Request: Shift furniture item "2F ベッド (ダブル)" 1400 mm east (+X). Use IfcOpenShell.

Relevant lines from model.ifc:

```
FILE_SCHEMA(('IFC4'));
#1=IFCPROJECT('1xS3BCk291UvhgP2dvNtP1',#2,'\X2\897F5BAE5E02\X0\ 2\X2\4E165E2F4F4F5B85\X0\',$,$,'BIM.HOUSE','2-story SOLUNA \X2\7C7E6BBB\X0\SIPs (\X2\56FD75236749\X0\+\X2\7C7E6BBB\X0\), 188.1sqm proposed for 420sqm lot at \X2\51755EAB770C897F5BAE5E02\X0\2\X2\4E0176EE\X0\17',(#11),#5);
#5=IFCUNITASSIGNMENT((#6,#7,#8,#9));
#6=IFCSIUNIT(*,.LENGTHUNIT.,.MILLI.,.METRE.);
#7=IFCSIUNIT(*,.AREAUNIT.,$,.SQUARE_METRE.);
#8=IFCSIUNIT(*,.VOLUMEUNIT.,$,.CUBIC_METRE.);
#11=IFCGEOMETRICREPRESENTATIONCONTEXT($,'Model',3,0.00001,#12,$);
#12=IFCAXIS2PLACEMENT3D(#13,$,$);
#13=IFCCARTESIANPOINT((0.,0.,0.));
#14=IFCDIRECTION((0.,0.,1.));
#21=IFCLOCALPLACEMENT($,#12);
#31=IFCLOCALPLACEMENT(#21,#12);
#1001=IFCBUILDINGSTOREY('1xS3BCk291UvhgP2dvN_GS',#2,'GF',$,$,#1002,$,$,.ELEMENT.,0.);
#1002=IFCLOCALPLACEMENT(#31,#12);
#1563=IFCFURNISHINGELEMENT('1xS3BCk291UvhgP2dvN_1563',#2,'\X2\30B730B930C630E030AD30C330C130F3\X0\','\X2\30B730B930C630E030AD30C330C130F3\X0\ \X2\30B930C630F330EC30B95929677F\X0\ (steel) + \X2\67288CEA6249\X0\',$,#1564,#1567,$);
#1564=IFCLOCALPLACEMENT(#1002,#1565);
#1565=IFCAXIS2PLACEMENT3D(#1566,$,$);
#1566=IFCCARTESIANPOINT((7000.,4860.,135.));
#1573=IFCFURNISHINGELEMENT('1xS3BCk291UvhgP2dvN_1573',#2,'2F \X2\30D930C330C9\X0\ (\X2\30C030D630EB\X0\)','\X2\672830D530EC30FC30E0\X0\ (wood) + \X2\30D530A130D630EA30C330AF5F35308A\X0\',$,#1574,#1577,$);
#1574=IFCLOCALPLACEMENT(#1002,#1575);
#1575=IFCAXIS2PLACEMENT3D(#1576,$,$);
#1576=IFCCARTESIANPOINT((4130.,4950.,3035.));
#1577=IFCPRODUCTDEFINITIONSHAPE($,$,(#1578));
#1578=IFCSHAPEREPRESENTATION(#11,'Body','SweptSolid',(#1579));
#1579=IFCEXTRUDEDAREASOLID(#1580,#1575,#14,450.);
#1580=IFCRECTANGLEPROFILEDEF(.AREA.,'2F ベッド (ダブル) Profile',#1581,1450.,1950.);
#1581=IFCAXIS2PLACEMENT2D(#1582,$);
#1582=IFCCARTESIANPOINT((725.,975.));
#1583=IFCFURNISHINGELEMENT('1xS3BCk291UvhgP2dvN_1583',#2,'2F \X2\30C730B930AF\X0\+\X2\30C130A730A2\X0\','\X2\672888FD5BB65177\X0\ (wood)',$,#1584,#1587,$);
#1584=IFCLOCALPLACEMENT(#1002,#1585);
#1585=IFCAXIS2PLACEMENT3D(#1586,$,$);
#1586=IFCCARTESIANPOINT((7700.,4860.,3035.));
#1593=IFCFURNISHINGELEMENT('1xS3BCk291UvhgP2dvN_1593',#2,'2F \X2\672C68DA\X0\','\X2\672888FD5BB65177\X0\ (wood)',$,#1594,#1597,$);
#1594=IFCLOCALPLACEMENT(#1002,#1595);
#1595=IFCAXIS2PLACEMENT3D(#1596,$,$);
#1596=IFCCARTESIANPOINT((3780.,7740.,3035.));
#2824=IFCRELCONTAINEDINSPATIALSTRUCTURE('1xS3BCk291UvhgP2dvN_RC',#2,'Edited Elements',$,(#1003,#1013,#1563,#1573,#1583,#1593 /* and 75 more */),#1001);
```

```python
import ifcopenshell
import ifcopenshell.api.geometry
import ifcopenshell.util.placement
import ifcopenshell.util.unit

model = ifcopenshell.open("model.ifc")
unit_scale = ifcopenshell.util.unit.calculate_unit_scale(model)

item = model.by_guid("1xS3BCk291UvhgP2dvN_1573")
matrix = ifcopenshell.util.placement.get_local_placement(item.ObjectPlacement)
matrix[0, 3] += 1.4 / unit_scale
ifcopenshell.api.geometry.edit_object_placement(model, product=item, matrix=matrix, is_si=False)

print(ifcopenshell.util.placement.get_local_placement(item.ObjectPlacement).round(3) + 0.0)

model.write("model-out.ifc")
```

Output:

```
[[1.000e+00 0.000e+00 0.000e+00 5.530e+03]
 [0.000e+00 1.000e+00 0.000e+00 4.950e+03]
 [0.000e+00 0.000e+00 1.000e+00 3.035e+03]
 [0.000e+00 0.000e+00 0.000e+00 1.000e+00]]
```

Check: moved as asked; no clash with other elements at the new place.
